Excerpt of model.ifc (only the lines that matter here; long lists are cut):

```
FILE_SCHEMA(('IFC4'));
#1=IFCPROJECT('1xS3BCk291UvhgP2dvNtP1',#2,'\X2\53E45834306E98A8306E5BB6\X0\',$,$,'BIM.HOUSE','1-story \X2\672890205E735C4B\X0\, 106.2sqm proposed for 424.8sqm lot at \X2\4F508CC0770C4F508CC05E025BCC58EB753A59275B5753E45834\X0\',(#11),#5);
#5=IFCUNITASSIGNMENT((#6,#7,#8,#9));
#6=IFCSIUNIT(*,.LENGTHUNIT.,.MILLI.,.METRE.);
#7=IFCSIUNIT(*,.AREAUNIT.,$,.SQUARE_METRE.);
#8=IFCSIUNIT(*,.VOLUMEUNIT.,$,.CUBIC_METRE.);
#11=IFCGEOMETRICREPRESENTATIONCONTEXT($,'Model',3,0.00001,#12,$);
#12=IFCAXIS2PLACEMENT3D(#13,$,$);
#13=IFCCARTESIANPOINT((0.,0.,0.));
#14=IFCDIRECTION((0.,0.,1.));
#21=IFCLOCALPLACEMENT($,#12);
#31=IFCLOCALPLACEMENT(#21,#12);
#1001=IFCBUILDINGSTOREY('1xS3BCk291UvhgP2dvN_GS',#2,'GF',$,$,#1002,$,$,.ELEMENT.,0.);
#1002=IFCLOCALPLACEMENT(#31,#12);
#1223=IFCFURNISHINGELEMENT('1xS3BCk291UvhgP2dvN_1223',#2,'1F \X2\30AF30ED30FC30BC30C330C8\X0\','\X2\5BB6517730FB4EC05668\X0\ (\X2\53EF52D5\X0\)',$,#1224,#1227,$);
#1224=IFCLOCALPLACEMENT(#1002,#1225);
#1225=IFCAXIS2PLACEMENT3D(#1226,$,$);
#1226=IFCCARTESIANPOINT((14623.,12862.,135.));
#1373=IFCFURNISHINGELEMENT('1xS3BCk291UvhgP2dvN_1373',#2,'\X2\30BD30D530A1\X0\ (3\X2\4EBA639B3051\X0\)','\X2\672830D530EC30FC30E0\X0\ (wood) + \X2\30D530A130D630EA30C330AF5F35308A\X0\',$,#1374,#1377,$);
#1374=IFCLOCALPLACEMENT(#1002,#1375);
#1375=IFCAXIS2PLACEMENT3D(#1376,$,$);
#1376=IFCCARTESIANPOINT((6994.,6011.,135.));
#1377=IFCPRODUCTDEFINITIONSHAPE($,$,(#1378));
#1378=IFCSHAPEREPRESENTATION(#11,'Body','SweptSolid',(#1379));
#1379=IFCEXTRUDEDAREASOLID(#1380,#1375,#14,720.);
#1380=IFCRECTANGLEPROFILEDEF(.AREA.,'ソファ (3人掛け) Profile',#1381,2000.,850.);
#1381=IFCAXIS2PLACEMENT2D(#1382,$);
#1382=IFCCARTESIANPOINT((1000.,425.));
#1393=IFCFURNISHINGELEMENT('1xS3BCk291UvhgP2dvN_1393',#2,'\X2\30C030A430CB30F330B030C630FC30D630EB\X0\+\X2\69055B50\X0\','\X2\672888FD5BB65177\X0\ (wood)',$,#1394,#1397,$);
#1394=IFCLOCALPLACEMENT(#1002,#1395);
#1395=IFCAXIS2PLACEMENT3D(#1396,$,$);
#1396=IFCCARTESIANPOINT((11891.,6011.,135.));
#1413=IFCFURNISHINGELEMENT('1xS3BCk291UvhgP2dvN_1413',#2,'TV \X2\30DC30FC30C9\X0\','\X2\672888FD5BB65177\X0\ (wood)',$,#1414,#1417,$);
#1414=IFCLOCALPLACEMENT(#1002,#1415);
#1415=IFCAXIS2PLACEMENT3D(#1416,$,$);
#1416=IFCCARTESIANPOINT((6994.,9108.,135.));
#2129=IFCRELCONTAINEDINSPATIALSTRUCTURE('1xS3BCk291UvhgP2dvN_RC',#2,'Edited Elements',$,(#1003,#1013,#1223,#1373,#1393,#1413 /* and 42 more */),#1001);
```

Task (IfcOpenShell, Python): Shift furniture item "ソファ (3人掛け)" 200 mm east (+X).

```python
import ifcopenshell
import ifcopenshell.api.geometry
import ifcopenshell.util.placement

model = ifcopenshell.open("model.ifc")

item = model.by_id(1373)
matrix = ifcopenshell.util.placement.get_local_placement(item.ObjectPlacement)
matrix[0, 3] += 200.0
ifcopenshell.api.geometry.edit_object_placement(model, product=item, matrix=matrix, is_si=False)

print(ifcopenshell.util.placement.get_local_placement(item.ObjectPlacement).round(3) + 0.0)

model.write("model_updated.ifc")
```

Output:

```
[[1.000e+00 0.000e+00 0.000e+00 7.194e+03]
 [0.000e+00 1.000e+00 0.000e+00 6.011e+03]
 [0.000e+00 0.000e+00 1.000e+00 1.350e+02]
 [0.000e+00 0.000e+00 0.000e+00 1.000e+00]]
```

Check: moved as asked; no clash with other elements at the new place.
